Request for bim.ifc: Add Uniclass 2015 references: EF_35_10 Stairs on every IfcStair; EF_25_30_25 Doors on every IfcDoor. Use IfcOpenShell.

First a look at what the model holds.

```python
import ifcopenshell

model = ifcopenshell.open("bim.ifc")
print(model.schema)
print("classifications:", [c.Name for c in model.by_type("IfcClassification")])
for ifc_class in ("IfcDoor", "IfcRoof", "IfcStair", "IfcWall", "IfcWindow"):
    print(ifc_class, len(model.by_type(ifc_class)))
```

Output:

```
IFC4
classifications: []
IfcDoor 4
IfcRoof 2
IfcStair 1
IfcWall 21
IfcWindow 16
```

```python
import ifcopenshell
import ifcopenshell.api.classification

model = ifcopenshell.open("bim.ifc")

system = ifcopenshell.api.classification.add_classification(model, classification="Uniclass 2015")

codes = {
    "IfcStair": ("EF_35_10", "Stairs"),
    "IfcDoor": ("EF_25_30_25", "Doors"),
}
for ifc_class, (code, name) in codes.items():
    products = model.by_type(ifc_class)
    ifcopenshell.api.classification.add_reference(
        model, products=products, classification=system, identification=code, name=name
    )
    print(code, len(products))

model.write("bim_v2.ifc")
```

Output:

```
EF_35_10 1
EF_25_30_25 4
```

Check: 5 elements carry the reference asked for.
